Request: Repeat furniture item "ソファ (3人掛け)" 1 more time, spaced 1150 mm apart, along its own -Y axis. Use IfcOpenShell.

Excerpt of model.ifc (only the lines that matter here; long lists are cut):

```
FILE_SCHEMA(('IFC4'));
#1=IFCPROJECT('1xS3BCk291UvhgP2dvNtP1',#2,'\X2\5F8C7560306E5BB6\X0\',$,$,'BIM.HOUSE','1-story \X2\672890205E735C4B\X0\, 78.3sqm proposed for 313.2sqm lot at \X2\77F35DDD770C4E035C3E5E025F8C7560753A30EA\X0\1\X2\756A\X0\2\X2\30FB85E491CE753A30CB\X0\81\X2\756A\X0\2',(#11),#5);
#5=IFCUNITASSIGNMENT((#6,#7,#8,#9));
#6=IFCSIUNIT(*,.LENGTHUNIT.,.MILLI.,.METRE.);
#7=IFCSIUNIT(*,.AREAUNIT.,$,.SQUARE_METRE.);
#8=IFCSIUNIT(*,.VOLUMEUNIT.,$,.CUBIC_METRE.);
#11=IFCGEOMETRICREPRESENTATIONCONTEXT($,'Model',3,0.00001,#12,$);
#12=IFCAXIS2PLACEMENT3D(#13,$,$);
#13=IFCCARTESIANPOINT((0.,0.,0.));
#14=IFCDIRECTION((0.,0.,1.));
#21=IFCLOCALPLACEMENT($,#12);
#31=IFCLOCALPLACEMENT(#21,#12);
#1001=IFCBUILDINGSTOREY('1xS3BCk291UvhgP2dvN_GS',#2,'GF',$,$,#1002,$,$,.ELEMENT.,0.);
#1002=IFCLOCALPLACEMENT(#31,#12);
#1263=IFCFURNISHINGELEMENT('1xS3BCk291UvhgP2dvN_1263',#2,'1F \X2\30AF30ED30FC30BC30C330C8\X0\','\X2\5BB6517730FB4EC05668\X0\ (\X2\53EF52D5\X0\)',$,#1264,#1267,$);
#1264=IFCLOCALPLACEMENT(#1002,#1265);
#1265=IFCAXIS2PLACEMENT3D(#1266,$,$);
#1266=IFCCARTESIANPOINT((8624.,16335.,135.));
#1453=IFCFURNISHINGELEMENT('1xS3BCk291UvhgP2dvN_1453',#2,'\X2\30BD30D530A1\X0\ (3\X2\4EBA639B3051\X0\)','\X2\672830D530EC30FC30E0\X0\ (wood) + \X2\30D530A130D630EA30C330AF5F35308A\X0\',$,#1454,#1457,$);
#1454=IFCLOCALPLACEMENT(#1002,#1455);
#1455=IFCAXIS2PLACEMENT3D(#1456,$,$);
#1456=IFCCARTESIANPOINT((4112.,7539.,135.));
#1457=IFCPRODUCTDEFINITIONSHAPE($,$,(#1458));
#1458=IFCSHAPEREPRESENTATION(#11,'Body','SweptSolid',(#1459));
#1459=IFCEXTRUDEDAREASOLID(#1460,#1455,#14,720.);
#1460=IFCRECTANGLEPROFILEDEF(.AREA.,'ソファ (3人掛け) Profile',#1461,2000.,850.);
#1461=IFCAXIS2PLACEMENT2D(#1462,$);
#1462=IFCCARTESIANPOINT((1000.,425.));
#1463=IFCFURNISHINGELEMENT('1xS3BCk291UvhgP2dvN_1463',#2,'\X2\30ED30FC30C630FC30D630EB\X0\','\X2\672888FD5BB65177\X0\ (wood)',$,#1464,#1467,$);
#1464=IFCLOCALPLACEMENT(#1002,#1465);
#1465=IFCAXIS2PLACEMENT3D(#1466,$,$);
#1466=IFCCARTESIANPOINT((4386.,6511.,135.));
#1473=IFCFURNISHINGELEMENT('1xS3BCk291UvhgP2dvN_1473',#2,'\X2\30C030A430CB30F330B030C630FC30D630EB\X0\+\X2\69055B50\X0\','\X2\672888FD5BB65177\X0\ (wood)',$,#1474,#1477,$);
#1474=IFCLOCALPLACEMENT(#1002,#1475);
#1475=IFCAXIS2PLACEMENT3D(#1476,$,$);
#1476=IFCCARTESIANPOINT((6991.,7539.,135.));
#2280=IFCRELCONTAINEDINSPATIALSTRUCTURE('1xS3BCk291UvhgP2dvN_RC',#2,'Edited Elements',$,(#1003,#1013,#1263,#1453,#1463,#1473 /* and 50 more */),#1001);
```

```python
import ifcopenshell
import ifcopenshell.api.geometry
import ifcopenshell.api.root
import ifcopenshell.util.element
import ifcopenshell.util.placement

model = ifcopenshell.open("model.ifc")


def reuse_history(source, copy):
    """copy_class also copies each property set's owner history, people and application; keep the originals."""
    for rel in copy.IsDefinedBy:
        if rel.is_a("IfcRelDefinesByProperties") and (history := rel.RelatingPropertyDefinition.OwnerHistory):
            rel.RelatingPropertyDefinition.OwnerHistory = source.OwnerHistory
            ifcopenshell.util.element.remove_deep2(model, history)


source = model.by_id(1453)
base = ifcopenshell.util.placement.get_local_placement(source.ObjectPlacement)
step = -base[:3, 1] * 1150.0

for i in range(1, 2):
    copy = ifcopenshell.api.root.copy_class(model, product=source)
    copy.Representation = ifcopenshell.util.element.copy_deep(
        model, source.Representation, exclude=["IfcGeometricRepresentationContext", "IfcRepresentationMap"]
    )
    reuse_history(source, copy)
    matrix = base.copy()
    matrix[:3, 3] += i * step
    print("added at", matrix[:3, 3].round(3) + 0.0)
    ifcopenshell.api.geometry.edit_object_placement(model, product=copy, matrix=matrix, is_si=False)

model.write("model_rev.ifc")
```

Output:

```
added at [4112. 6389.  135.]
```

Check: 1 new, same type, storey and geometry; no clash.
